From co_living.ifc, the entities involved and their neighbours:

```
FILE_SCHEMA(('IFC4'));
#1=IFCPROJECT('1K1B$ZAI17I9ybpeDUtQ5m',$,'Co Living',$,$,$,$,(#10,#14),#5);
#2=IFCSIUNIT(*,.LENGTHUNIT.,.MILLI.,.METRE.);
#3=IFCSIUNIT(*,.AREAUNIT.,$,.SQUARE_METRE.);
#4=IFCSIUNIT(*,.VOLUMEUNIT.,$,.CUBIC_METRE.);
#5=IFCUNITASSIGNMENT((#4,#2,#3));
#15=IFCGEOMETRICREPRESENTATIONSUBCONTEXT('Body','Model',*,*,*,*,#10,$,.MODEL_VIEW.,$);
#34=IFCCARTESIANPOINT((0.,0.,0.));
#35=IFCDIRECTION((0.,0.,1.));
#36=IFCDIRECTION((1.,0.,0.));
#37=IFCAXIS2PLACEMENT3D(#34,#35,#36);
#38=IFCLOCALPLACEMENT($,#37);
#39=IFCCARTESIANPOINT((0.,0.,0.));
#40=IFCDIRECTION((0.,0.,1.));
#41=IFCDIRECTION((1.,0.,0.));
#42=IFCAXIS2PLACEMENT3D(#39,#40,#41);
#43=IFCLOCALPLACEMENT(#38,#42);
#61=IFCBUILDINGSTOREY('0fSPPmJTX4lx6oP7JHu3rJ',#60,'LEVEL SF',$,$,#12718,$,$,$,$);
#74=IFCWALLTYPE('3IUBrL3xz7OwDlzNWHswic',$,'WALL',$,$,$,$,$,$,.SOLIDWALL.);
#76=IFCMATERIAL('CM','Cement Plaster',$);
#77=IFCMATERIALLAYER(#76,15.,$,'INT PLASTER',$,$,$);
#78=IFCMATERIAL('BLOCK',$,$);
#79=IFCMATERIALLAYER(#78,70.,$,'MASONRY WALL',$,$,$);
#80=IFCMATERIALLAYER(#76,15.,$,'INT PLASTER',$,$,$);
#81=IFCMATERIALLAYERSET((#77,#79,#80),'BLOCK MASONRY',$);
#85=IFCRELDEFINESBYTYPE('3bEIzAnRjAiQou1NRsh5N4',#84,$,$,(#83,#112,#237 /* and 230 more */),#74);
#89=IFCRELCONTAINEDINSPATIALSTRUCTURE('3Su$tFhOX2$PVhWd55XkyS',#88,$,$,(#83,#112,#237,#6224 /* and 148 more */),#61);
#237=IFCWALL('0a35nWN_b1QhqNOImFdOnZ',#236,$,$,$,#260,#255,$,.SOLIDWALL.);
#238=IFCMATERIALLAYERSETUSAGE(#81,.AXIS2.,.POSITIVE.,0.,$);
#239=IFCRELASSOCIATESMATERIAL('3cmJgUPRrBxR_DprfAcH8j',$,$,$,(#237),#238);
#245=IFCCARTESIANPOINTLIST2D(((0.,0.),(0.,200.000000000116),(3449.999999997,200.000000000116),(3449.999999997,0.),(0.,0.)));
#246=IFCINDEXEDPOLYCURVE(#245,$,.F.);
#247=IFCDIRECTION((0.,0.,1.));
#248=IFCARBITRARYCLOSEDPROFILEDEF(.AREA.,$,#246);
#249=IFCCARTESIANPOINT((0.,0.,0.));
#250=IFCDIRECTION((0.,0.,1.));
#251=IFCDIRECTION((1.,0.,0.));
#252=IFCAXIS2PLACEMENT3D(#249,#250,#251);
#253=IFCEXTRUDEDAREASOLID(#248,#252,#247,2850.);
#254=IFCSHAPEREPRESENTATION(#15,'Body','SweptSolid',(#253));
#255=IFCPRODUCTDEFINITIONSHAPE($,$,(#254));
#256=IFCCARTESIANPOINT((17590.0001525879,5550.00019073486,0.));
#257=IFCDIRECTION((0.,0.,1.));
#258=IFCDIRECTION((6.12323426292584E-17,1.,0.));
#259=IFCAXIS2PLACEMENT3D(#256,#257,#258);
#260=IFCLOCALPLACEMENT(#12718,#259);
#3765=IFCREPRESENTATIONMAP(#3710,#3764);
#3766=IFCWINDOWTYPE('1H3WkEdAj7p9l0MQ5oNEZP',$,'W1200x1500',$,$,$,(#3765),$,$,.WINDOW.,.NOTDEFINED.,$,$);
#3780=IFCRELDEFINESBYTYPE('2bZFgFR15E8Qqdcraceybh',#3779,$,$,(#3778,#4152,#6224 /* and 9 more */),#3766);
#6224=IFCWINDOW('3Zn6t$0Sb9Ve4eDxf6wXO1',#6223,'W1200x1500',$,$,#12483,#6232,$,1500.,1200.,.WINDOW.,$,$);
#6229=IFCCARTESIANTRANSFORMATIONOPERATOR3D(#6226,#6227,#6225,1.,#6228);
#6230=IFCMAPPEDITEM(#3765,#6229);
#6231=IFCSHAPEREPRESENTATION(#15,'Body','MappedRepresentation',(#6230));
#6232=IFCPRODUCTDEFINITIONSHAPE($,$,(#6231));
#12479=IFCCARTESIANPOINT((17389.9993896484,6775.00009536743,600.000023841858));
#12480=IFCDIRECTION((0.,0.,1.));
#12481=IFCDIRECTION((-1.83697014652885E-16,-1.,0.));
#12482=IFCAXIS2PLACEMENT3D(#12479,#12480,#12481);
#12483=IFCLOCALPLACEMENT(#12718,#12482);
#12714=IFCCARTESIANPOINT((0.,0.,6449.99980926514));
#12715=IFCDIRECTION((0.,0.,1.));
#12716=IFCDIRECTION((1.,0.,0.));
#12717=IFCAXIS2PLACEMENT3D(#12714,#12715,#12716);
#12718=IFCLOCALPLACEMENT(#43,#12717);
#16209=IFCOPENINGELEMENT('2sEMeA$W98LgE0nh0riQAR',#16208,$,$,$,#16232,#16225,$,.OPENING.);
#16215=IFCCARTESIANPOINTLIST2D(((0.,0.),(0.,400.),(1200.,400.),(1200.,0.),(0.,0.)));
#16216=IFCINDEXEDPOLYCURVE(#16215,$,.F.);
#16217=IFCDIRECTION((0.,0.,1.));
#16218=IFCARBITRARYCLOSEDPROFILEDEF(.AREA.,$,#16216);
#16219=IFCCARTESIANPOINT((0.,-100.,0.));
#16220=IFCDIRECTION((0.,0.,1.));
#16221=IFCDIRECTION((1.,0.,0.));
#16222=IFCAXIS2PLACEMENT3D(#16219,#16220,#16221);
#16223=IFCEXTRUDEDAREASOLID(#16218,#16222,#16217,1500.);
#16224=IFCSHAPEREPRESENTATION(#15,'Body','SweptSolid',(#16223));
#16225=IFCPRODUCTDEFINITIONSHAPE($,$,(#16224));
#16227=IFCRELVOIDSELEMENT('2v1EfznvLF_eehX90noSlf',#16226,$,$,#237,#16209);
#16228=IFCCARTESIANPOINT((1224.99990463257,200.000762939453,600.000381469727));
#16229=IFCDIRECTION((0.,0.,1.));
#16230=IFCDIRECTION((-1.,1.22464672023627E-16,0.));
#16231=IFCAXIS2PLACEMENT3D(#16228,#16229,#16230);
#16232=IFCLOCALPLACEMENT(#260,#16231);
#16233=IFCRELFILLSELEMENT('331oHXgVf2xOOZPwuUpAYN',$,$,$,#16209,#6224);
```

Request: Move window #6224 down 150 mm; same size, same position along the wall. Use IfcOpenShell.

```python
import numpy as np
import ifcopenshell
import ifcopenshell.api.geometry
import ifcopenshell.util.placement
import ifcopenshell.util.unit

model = ifcopenshell.open("co_living.ifc")
unit_scale = ifcopenshell.util.unit.calculate_unit_scale(model)

window = model.by_guid("3Zn6t$0Sb9Ve4eDxf6wXO1")
opening = window.FillsVoids[0].RelatingOpeningElement
dz = -150.0

shift = np.array([0.0, 0.0, dz])
# The window is not placed relative to its opening, so move both.
for product in (opening, window):
    matrix = ifcopenshell.util.placement.get_local_placement(product.ObjectPlacement)
    matrix[:3, 3] += shift
    ifcopenshell.api.geometry.edit_object_placement(model, product=product, matrix=matrix, is_si=False)

print(f"moved by {dz * unit_scale:+.3f} m")

model.write("co_living_updated.ifc")
```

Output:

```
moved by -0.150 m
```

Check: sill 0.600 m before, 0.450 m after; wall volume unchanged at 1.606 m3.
